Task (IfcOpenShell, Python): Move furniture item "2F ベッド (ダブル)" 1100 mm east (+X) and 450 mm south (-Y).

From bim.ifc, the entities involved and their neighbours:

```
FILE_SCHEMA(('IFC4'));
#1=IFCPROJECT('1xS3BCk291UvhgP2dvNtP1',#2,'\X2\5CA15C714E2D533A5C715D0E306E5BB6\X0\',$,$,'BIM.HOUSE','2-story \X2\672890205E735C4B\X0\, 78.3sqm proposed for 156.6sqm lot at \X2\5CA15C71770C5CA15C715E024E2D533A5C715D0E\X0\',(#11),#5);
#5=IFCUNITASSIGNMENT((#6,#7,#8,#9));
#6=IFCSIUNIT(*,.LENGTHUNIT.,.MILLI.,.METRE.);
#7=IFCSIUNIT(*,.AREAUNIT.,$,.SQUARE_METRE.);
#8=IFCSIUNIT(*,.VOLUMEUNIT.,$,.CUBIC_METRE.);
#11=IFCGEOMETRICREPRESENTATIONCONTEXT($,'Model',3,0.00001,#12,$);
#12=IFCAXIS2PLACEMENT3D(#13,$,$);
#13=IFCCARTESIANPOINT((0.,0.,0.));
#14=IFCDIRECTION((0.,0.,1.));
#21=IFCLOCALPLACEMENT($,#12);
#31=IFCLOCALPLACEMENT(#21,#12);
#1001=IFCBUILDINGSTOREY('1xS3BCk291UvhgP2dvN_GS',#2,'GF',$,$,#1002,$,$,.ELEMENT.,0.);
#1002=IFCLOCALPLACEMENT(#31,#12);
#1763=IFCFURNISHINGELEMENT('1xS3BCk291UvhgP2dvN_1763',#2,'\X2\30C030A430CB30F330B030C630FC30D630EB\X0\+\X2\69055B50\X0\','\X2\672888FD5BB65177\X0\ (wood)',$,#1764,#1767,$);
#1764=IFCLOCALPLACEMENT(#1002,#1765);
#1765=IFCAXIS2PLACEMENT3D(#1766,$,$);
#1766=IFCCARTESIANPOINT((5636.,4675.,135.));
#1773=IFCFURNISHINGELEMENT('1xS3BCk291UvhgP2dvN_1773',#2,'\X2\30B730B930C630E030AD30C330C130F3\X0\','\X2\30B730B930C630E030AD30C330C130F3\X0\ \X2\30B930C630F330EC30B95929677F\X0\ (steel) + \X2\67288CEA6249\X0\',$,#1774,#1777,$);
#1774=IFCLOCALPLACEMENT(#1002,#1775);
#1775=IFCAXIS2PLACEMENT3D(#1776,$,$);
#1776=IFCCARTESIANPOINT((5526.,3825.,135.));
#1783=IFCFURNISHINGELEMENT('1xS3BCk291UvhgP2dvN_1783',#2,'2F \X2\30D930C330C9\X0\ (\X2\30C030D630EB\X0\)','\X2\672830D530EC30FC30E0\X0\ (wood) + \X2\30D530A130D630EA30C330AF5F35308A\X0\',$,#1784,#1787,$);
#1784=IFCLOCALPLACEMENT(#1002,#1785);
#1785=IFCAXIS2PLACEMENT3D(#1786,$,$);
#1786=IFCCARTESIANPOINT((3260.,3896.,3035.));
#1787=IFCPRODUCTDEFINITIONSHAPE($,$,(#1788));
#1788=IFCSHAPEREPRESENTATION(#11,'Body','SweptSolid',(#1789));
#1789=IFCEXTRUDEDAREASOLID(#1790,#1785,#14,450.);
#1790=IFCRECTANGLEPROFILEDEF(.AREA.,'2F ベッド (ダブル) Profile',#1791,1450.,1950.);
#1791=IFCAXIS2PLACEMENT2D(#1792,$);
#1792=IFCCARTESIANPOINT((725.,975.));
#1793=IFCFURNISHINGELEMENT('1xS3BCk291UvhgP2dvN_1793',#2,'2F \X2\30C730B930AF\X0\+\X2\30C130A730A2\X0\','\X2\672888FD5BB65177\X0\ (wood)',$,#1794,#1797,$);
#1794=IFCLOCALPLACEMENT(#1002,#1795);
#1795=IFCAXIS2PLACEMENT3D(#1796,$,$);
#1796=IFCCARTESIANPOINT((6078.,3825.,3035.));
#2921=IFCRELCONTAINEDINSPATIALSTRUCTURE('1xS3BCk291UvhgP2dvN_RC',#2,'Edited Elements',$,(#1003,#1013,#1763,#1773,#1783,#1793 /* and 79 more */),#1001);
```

```python
import ifcopenshell
import ifcopenshell.api.geometry
import ifcopenshell.util.placement
import ifcopenshell.util.unit

model = ifcopenshell.open("bim.ifc")
unit_scale = ifcopenshell.util.unit.calculate_unit_scale(model)

item = model.by_guid("1xS3BCk291UvhgP2dvN_1783")
matrix = ifcopenshell.util.placement.get_local_placement(item.ObjectPlacement)
matrix[0, 3] += 1.1 / unit_scale
matrix[1, 3] -= 0.45 / unit_scale
ifcopenshell.api.geometry.edit_object_placement(model, product=item, matrix=matrix, is_si=False)

print(ifcopenshell.util.placement.get_local_placement(item.ObjectPlacement).round(3) + 0.0)

model.write("bim_rev.ifc")
```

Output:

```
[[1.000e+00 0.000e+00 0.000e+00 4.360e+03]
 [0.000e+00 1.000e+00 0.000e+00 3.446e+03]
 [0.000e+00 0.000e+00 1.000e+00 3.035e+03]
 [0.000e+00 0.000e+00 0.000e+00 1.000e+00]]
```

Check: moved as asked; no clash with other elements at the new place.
